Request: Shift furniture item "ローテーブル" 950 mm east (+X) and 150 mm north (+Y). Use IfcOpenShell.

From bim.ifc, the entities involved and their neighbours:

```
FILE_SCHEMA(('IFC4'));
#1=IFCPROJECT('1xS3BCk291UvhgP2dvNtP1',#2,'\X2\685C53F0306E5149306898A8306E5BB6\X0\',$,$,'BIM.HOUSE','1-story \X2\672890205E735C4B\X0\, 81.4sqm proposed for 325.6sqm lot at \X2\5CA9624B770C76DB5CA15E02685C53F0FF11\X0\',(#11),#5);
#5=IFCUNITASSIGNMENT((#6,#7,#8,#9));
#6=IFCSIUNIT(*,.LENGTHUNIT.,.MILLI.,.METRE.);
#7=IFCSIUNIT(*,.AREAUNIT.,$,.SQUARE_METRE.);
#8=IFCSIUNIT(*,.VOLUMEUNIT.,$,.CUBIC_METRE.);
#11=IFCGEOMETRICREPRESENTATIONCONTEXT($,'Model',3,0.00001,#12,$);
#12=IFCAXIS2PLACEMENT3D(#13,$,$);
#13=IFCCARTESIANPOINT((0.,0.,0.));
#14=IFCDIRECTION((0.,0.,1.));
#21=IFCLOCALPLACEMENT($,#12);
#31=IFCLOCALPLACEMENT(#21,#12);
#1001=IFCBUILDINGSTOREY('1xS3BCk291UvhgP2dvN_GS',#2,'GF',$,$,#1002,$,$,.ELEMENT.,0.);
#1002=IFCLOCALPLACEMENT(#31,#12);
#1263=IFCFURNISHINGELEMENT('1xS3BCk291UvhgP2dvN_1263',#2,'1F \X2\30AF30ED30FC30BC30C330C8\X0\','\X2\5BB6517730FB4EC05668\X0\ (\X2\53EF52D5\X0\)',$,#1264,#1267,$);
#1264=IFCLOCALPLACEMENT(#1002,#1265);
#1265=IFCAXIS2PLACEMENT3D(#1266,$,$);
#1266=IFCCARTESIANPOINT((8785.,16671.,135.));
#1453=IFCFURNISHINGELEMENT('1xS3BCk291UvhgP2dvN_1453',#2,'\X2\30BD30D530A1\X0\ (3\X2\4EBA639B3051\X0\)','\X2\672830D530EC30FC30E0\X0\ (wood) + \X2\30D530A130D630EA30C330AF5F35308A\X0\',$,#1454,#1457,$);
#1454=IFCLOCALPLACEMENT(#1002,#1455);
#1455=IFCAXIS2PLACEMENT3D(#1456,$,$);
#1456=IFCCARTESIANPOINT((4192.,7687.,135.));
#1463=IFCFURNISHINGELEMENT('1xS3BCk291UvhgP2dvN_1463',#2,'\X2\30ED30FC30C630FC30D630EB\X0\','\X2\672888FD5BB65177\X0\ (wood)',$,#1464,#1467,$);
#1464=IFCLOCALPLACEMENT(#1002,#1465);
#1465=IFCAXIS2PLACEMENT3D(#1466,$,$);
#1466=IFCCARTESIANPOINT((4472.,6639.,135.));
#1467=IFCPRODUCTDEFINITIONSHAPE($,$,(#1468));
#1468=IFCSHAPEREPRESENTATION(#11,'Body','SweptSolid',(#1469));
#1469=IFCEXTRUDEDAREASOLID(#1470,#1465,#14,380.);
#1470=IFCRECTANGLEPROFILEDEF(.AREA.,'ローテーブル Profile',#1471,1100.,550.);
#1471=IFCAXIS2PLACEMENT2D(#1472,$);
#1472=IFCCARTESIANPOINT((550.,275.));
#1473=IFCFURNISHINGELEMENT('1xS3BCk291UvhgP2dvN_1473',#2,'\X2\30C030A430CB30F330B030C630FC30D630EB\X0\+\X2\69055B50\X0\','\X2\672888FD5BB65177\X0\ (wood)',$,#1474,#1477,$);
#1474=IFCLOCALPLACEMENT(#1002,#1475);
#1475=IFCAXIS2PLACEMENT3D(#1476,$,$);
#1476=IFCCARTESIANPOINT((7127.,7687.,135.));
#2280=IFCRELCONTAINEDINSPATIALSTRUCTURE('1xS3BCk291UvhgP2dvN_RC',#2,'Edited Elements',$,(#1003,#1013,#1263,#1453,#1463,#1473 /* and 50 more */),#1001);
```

```python
import ifcopenshell
import ifcopenshell.api.geometry
import ifcopenshell.util.placement
import ifcopenshell.util.unit

model = ifcopenshell.open("bim.ifc")
unit_scale = ifcopenshell.util.unit.calculate_unit_scale(model)

item = model.by_guid("1xS3BCk291UvhgP2dvN_1463")
matrix = ifcopenshell.util.placement.get_local_placement(item.ObjectPlacement)
matrix[0, 3] += 0.95 / unit_scale
matrix[1, 3] += 0.15 / unit_scale
ifcopenshell.api.geometry.edit_object_placement(model, product=item, matrix=matrix, is_si=False)

print(ifcopenshell.util.placement.get_local_placement(item.ObjectPlacement).round(3) + 0.0)

model.write("bim_edited.ifc")
```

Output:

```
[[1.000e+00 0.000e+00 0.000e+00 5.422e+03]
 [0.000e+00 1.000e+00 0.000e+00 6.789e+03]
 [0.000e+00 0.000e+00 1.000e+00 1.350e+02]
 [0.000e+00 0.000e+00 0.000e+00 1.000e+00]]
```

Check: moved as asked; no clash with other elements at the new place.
